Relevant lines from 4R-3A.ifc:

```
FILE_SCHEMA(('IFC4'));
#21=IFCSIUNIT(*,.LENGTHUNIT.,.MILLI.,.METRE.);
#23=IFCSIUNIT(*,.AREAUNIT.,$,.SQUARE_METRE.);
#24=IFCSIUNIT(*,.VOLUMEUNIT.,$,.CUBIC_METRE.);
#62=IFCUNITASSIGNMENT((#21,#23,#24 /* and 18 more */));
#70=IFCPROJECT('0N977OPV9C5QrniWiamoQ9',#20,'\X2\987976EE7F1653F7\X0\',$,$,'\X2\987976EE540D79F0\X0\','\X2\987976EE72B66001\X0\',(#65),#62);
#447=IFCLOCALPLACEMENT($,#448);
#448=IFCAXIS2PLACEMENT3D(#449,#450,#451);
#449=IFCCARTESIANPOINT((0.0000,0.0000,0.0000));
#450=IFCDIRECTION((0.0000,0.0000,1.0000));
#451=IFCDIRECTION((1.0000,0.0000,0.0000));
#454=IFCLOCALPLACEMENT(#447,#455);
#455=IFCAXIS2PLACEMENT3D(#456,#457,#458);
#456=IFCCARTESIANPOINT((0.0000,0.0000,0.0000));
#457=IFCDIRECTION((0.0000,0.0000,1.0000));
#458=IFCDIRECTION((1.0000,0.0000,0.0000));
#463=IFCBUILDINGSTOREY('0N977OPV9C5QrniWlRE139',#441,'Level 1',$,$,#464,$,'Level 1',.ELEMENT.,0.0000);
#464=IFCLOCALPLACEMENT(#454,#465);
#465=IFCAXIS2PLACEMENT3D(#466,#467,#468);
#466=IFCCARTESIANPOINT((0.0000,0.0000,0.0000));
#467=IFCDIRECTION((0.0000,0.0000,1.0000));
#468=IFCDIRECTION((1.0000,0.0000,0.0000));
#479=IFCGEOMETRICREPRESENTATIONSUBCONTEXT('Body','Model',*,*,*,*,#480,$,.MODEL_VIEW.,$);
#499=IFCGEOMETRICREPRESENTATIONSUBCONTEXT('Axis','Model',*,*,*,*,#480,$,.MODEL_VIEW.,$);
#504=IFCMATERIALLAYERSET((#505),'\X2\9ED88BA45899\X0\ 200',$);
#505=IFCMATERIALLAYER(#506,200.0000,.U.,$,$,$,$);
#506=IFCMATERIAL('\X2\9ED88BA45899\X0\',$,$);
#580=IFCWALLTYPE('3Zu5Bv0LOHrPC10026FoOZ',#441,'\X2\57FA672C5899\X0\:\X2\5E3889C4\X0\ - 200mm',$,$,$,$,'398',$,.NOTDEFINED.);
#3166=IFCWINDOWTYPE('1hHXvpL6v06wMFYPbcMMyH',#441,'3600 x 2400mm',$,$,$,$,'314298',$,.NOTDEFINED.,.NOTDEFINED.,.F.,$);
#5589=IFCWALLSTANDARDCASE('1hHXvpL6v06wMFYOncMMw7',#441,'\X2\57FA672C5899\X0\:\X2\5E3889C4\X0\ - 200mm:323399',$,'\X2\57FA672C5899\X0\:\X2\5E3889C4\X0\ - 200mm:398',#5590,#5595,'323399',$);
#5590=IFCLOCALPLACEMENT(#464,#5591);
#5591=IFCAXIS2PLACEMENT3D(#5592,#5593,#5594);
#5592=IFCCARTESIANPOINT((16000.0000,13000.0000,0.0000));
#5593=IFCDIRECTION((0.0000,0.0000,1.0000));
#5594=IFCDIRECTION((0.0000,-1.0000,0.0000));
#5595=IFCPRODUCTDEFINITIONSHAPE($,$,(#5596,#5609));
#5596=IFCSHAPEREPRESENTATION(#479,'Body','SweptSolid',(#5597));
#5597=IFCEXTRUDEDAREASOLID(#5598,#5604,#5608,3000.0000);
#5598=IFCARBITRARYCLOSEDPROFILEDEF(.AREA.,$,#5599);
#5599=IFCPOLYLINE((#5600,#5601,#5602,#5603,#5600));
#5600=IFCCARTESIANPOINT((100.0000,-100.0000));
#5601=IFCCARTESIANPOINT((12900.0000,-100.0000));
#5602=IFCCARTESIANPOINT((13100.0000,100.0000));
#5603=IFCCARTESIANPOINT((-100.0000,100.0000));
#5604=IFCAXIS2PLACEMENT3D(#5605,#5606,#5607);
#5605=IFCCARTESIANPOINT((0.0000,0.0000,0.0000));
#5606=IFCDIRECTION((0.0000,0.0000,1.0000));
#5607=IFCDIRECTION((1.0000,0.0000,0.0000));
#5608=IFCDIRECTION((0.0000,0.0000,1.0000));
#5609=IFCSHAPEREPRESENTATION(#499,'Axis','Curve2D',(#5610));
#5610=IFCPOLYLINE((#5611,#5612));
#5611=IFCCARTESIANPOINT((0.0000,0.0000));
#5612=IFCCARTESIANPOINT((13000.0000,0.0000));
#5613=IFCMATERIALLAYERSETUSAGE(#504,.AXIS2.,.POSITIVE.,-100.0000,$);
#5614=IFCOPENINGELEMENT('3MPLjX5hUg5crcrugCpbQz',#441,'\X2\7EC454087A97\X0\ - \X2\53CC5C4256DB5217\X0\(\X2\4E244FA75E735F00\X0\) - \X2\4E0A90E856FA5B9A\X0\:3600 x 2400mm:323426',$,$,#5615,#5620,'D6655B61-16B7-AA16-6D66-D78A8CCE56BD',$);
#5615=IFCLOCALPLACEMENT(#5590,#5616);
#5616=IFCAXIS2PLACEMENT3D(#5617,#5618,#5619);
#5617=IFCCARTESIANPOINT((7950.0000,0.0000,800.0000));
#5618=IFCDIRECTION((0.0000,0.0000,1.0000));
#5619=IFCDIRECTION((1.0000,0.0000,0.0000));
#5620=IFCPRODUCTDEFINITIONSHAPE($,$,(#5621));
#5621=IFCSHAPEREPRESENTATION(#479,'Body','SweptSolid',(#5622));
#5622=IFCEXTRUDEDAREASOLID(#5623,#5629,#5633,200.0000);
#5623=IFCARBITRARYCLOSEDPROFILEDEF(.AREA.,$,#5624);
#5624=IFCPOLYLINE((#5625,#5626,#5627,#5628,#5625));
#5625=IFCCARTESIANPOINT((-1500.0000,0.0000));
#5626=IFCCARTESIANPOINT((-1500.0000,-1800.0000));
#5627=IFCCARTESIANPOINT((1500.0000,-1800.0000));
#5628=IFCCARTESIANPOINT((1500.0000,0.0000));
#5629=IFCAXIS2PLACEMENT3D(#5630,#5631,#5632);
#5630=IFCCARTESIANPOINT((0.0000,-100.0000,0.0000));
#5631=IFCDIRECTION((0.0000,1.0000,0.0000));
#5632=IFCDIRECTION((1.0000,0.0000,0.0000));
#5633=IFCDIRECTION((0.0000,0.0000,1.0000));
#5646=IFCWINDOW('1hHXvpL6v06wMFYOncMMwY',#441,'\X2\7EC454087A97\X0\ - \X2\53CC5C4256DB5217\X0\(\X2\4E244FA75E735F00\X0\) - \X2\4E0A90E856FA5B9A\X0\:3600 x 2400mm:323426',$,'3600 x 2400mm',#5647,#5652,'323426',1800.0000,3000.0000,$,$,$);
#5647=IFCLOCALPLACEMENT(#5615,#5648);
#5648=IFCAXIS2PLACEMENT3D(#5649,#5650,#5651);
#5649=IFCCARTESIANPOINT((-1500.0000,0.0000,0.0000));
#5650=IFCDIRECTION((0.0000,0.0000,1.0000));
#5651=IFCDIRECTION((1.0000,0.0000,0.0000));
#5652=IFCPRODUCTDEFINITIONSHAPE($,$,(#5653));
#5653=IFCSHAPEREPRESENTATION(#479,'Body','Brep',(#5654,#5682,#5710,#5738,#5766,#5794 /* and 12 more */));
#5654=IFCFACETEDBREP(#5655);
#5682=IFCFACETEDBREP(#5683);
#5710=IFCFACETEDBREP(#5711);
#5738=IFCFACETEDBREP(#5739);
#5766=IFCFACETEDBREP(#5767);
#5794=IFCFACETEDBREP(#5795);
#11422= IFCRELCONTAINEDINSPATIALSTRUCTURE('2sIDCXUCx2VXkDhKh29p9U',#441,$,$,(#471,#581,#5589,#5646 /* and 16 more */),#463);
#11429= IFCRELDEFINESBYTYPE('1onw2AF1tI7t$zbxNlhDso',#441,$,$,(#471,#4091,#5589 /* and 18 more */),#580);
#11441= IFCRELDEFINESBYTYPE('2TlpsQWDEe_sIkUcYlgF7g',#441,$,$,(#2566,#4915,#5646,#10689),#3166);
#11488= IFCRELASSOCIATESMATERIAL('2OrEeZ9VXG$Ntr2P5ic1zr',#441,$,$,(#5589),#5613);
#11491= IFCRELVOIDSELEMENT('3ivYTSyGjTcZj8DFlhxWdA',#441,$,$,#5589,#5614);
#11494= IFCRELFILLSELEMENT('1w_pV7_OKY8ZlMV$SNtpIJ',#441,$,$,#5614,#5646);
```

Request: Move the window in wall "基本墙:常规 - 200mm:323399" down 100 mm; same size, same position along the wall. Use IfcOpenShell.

```python
import numpy as np
import ifcopenshell
import ifcopenshell.api.geometry
import ifcopenshell.util.placement
import ifcopenshell.util.unit

model = ifcopenshell.open("4R-3A.ifc")
unit_scale = ifcopenshell.util.unit.calculate_unit_scale(model)

window = model.by_guid("1hHXvpL6v06wMFYOncMMwY")
opening = window.FillsVoids[0].RelatingOpeningElement
dz = -100.0

shift = np.array([0.0, 0.0, dz])
# The window is placed relative to its opening, so it follows when the opening moves.
matrix = ifcopenshell.util.placement.get_local_placement(opening.ObjectPlacement)
matrix[:3, 3] += shift
ifcopenshell.api.geometry.edit_object_placement(
    model, product=opening, matrix=matrix, is_si=False, should_transform_children=True
)

print(f"moved by {dz * unit_scale:+.3f} m")

model.write("4R-3A_rev.ifc")
```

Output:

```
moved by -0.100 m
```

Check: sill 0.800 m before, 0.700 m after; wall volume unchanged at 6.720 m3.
